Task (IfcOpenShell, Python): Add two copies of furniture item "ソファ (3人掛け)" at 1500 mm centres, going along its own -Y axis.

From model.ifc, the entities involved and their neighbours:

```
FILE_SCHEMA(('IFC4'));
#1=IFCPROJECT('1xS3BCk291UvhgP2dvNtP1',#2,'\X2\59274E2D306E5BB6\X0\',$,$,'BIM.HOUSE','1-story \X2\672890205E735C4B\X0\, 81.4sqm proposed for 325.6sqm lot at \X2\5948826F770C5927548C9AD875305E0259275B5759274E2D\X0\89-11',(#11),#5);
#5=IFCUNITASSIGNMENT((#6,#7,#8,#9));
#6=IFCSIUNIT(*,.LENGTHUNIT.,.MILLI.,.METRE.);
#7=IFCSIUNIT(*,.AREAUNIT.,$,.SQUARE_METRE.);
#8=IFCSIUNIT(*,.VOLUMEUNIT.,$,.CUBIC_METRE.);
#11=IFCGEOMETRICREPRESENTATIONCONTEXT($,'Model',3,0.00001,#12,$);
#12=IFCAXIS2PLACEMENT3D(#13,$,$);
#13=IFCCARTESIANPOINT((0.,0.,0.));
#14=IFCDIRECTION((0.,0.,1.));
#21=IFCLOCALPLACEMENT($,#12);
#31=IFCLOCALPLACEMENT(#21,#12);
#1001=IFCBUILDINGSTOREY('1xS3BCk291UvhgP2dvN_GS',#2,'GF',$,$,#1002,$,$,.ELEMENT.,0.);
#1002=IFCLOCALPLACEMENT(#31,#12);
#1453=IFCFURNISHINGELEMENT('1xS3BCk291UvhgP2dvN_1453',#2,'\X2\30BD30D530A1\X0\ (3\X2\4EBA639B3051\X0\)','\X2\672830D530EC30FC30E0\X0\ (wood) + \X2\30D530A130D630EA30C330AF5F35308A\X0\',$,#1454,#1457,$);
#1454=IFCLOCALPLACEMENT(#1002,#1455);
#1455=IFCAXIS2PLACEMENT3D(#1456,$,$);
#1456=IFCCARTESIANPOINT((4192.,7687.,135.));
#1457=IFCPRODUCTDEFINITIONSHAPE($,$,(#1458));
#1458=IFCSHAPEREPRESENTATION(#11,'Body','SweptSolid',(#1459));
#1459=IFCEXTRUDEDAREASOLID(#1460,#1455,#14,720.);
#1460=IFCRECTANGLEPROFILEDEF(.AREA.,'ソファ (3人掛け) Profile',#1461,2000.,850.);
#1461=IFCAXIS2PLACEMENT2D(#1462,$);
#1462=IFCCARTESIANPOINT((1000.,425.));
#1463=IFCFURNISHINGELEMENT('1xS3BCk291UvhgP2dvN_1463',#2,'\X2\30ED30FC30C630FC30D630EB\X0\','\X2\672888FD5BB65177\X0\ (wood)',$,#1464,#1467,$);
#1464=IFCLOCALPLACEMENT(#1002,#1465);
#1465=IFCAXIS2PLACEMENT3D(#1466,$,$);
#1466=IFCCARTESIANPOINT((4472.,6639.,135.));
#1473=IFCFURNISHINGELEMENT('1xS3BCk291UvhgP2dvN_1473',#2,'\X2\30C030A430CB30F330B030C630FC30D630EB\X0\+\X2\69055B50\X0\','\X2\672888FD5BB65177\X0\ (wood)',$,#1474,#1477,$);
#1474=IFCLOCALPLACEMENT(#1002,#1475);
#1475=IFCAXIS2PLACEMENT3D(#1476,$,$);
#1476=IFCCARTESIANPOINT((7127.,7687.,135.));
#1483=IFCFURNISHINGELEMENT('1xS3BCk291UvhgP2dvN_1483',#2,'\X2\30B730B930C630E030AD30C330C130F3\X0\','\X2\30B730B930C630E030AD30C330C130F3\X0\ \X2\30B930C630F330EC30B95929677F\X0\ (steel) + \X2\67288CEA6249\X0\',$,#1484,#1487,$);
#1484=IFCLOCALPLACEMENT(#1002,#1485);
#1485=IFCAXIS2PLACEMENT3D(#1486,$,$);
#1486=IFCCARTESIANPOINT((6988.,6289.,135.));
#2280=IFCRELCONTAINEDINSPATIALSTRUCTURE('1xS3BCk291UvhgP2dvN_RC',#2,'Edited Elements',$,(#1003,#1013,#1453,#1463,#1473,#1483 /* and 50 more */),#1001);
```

```python
import ifcopenshell
import ifcopenshell.api.geometry
import ifcopenshell.api.root
import ifcopenshell.util.element
import ifcopenshell.util.placement

model = ifcopenshell.open("model.ifc")


def reuse_history(source, copy):
    """copy_class also copies each property set's owner history, people and application; keep the originals."""
    for rel in copy.IsDefinedBy:
        if rel.is_a("IfcRelDefinesByProperties") and (history := rel.RelatingPropertyDefinition.OwnerHistory):
            rel.RelatingPropertyDefinition.OwnerHistory = source.OwnerHistory
            ifcopenshell.util.element.remove_deep2(model, history)


source = model.by_id(1453)
base = ifcopenshell.util.placement.get_local_placement(source.ObjectPlacement)
step = -base[:3, 1] * 1500.0

for i in range(1, 3):
    copy = ifcopenshell.api.root.copy_class(model, product=source)
    copy.Representation = ifcopenshell.util.element.copy_deep(
        model, source.Representation, exclude=["IfcGeometricRepresentationContext", "IfcRepresentationMap"]
    )
    reuse_history(source, copy)
    matrix = base.copy()
    matrix[:3, 3] += i * step
    print("added at", matrix[:3, 3].round(3) + 0.0)
    ifcopenshell.api.geometry.edit_object_placement(model, product=copy, matrix=matrix, is_si=False)

model.write("model_edited.ifc")
```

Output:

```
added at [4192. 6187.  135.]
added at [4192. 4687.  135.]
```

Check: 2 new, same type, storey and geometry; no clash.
